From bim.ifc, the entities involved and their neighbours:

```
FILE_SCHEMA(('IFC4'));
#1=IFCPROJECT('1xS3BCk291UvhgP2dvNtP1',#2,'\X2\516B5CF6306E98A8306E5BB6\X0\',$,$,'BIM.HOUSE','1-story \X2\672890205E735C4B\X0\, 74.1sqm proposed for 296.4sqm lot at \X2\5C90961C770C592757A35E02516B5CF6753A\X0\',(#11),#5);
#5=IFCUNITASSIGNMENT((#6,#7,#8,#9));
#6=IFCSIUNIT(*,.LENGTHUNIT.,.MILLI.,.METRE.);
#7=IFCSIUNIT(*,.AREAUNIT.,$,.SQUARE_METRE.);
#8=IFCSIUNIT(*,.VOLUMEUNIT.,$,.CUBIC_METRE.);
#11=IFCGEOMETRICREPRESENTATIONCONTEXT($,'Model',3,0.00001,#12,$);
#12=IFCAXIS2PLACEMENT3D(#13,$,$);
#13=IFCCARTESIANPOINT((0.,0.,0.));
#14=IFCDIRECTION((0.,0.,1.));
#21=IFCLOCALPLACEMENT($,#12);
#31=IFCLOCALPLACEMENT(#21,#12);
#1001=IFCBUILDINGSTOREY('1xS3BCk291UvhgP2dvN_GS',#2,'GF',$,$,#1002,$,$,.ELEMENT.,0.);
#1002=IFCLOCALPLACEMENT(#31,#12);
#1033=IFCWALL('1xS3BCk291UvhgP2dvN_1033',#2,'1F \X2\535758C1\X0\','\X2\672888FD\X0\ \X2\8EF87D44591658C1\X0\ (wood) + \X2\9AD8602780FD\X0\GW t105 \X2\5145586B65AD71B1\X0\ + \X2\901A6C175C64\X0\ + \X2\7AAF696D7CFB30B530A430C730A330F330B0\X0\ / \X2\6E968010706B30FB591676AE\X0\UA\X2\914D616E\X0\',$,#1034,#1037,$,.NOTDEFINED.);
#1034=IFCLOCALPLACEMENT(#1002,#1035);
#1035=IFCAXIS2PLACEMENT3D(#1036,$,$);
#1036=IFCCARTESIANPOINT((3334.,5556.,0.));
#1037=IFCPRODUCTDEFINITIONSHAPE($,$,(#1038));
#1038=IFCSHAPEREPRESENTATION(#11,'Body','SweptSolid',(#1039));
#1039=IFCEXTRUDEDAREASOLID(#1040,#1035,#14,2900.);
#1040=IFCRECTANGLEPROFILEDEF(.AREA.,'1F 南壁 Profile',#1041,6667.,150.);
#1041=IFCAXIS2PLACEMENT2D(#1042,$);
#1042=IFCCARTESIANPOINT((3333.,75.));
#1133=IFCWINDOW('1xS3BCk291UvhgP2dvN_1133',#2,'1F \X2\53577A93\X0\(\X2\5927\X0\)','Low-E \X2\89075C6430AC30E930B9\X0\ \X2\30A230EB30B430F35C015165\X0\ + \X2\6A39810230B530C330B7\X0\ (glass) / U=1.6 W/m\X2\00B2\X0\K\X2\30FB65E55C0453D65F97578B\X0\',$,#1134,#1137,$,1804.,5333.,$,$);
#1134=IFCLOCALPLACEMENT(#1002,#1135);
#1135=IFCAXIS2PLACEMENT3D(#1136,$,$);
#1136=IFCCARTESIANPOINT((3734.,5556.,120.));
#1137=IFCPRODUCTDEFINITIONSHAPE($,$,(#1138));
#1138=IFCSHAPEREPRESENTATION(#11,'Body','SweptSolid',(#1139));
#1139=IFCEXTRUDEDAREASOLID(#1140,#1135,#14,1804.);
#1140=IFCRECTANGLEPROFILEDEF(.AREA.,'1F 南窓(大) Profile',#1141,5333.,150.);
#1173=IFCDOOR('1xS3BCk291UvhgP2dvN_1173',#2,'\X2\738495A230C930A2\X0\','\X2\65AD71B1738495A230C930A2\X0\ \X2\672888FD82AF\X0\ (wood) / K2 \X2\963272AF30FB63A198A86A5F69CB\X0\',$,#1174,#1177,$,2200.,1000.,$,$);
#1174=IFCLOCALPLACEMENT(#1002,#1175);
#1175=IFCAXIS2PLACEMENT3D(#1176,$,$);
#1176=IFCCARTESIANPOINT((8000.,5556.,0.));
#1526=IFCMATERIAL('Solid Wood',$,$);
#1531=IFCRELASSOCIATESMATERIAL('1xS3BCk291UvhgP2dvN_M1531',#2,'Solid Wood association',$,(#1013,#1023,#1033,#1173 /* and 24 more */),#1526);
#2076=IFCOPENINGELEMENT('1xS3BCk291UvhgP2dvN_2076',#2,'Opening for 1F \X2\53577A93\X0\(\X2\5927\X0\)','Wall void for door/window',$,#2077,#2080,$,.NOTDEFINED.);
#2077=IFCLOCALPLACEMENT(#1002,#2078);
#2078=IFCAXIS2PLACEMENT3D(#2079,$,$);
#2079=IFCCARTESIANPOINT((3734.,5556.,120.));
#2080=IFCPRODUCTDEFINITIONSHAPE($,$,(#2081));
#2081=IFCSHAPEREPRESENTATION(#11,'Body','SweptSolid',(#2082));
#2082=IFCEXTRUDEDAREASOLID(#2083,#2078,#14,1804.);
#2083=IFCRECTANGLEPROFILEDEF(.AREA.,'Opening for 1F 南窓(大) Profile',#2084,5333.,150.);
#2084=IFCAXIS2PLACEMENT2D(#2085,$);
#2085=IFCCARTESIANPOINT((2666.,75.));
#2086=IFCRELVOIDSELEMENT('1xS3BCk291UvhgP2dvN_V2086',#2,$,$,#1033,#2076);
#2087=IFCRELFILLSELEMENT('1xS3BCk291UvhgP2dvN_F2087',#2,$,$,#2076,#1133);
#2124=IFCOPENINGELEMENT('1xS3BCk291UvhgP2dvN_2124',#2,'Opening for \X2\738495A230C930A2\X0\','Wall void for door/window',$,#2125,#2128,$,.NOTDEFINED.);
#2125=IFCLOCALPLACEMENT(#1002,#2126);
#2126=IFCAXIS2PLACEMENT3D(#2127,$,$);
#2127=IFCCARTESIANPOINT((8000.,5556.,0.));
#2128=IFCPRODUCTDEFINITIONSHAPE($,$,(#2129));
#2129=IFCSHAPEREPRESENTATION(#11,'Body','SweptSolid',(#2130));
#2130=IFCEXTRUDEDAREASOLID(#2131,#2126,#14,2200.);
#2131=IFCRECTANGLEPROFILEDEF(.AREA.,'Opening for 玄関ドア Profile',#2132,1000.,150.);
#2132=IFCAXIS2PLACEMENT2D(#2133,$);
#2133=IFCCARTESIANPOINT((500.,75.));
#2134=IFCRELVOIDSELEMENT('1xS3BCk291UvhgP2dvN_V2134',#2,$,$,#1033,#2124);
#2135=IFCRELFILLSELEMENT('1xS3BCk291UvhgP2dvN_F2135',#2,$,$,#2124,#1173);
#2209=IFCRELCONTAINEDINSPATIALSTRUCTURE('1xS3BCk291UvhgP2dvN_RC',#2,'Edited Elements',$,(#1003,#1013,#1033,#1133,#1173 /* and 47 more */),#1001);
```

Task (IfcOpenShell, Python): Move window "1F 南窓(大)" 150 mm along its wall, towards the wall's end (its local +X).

```python
import ifcopenshell
import ifcopenshell.api.geometry
import ifcopenshell.util.placement

model = ifcopenshell.open("bim.ifc")

window = model.by_guid("1xS3BCk291UvhgP2dvN_1133")
opening = window.FillsVoids[0].RelatingOpeningElement
wall = opening.VoidsElements[0].RelatingBuildingElement

wall_matrix = ifcopenshell.util.placement.get_local_placement(wall.ObjectPlacement)
shift = wall_matrix[:3, 0] * 150.0
before = ifcopenshell.util.placement.get_local_placement(window.ObjectPlacement)[:3, 3].copy()

# The window is not placed relative to its opening, so move both.
for product in (opening, window):
    matrix = ifcopenshell.util.placement.get_local_placement(product.ObjectPlacement)
    matrix[:3, 3] += shift
    ifcopenshell.api.geometry.edit_object_placement(model, product=product, matrix=matrix, is_si=False)

after = ifcopenshell.util.placement.get_local_placement(window.ObjectPlacement)[:3, 3]
print("window moved by", (after - before).round(3) + 0.0)

model.write("bim_updated.ifc")
```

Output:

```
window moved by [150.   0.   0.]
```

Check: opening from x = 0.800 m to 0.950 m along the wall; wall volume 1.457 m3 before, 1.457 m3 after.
